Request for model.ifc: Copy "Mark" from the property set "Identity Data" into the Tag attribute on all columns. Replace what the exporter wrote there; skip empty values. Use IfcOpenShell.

First a look at what the model holds.

```python
import ifcopenshell
import ifcopenshell.util.element

model = ifcopenshell.open("model.ifc")
print(model.schema)
columns = model.by_type("IfcColumn")
print(len(columns), "columns")
for e in columns[:8]:
    source = ifcopenshell.util.element.get_pset(e, "Identity Data", "Mark")
    target = e.Tag
    print(e.id(), repr(source), repr(target), sep=" | ")
```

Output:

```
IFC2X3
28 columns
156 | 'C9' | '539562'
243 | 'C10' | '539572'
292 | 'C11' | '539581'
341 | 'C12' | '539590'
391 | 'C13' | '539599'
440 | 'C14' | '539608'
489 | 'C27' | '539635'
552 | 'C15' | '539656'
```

```python
import ifcopenshell
import ifcopenshell.util.element

model = ifcopenshell.open("model.ifc")

count = 0
for e in model.by_type("IfcColumn"):
    value = ifcopenshell.util.element.get_pset(e, "Identity Data", "Mark")
    current = e.Tag
    if not value or not value.strip() or current == value:
        continue
    e.Tag = value
    count += 1

print(count, "columns updated")

model.write("model_updated.ifc")
```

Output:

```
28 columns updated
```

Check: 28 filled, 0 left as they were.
